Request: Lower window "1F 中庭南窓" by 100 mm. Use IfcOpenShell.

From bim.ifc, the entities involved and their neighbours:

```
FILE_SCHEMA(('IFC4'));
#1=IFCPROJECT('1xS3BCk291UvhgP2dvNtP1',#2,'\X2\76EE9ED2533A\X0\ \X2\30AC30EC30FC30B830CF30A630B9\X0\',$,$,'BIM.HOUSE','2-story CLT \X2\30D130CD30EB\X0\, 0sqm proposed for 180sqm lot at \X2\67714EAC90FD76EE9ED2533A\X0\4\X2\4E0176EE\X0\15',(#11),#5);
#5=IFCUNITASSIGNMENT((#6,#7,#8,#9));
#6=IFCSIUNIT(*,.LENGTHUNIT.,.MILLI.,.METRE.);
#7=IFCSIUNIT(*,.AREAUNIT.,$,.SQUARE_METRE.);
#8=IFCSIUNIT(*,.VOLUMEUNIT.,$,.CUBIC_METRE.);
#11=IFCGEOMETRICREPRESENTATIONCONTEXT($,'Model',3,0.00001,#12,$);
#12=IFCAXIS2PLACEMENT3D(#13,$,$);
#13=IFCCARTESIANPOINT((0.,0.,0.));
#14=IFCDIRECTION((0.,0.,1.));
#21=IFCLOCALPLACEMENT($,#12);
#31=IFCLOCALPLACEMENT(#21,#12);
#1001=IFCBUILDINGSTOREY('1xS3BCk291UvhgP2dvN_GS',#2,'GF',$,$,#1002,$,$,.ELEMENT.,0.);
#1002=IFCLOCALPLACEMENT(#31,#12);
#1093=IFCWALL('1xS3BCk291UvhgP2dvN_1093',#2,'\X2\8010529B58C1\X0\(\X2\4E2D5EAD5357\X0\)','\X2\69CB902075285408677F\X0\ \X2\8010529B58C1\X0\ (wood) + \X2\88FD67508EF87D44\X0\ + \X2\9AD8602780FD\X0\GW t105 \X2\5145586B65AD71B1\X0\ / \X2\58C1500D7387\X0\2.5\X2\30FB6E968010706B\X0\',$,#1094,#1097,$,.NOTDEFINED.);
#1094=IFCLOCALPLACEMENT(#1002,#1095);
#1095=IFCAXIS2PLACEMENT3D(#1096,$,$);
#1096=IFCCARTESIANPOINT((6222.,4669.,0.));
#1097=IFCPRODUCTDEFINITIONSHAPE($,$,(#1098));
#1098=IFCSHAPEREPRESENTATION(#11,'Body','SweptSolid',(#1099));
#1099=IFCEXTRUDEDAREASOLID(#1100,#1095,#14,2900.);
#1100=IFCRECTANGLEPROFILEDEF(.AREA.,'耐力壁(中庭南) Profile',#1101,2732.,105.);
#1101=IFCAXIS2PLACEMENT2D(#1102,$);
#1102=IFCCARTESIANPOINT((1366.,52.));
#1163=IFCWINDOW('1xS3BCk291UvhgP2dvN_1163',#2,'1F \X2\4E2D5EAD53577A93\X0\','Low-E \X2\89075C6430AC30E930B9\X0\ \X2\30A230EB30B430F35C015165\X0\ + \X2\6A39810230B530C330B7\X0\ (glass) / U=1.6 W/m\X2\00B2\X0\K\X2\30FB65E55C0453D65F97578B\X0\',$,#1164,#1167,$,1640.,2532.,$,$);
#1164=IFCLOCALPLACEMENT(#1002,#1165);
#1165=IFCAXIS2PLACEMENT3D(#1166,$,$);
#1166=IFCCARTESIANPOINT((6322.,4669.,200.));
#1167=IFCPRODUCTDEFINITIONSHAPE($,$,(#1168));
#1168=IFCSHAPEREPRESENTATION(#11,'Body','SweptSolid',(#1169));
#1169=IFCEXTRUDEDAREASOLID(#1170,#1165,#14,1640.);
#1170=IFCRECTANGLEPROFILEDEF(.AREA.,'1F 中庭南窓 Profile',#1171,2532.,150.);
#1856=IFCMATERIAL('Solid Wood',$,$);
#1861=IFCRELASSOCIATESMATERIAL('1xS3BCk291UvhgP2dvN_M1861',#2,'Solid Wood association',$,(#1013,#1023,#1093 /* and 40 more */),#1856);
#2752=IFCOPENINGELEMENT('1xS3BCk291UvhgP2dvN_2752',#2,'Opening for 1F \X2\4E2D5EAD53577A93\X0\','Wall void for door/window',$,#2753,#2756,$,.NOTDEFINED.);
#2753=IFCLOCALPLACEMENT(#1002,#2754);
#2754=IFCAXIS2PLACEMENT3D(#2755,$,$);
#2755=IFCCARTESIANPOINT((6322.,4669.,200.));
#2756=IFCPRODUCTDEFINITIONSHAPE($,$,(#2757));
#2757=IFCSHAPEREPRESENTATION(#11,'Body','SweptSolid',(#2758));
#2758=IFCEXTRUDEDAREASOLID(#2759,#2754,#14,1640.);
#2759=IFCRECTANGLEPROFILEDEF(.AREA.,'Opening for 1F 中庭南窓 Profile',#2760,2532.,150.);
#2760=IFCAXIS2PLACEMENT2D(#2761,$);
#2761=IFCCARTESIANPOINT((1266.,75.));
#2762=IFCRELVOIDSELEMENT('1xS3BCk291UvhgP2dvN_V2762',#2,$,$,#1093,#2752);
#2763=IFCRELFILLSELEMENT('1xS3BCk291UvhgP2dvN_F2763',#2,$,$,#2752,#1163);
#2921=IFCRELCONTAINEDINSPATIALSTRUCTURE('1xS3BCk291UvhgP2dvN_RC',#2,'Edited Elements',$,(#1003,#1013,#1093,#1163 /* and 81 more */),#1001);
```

```python
import numpy as np
import ifcopenshell
import ifcopenshell.api.geometry
import ifcopenshell.util.placement
import ifcopenshell.util.unit

model = ifcopenshell.open("bim.ifc")
unit_scale = ifcopenshell.util.unit.calculate_unit_scale(model)

window = model.by_guid("1xS3BCk291UvhgP2dvN_1163")
opening = window.FillsVoids[0].RelatingOpeningElement
dz = -0.1 / unit_scale

shift = np.array([0.0, 0.0, dz])
# The window is not placed relative to its opening, so move both.
for product in (opening, window):
    matrix = ifcopenshell.util.placement.get_local_placement(product.ObjectPlacement)
    matrix[:3, 3] += shift
    ifcopenshell.api.geometry.edit_object_placement(model, product=product, matrix=matrix, is_si=False)

print(f"moved by {dz * unit_scale:+.3f} m")

model.write("bim_updated.ifc")
```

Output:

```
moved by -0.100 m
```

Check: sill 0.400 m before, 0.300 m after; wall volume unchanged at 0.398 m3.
